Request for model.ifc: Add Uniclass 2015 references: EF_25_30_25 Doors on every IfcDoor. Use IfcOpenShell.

First a look at what the model holds.

```python
import ifcopenshell

model = ifcopenshell.open("model.ifc")
print(model.schema)
print("classifications:", [c.Name for c in model.by_type("IfcClassification")])
for ifc_class in ("IfcDoor", "IfcRoof", "IfcStair", "IfcWall", "IfcWindow"):
    print(ifc_class, len(model.by_type(ifc_class)))
```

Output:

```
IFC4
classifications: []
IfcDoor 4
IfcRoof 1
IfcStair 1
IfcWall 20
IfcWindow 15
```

```python
import ifcopenshell
import ifcopenshell.api.classification

model = ifcopenshell.open("model.ifc")

system = ifcopenshell.api.classification.add_classification(model, classification="Uniclass 2015")

codes = {
    "IfcDoor": ("EF_25_30_25", "Doors"),
}
for ifc_class, (code, name) in codes.items():
    products = model.by_type(ifc_class)
    ifcopenshell.api.classification.add_reference(
        model, products=products, classification=system, identification=code, name=name
    )
    print(code, len(products))

model.write("model-out.ifc")
```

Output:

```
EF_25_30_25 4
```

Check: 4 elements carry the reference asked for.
